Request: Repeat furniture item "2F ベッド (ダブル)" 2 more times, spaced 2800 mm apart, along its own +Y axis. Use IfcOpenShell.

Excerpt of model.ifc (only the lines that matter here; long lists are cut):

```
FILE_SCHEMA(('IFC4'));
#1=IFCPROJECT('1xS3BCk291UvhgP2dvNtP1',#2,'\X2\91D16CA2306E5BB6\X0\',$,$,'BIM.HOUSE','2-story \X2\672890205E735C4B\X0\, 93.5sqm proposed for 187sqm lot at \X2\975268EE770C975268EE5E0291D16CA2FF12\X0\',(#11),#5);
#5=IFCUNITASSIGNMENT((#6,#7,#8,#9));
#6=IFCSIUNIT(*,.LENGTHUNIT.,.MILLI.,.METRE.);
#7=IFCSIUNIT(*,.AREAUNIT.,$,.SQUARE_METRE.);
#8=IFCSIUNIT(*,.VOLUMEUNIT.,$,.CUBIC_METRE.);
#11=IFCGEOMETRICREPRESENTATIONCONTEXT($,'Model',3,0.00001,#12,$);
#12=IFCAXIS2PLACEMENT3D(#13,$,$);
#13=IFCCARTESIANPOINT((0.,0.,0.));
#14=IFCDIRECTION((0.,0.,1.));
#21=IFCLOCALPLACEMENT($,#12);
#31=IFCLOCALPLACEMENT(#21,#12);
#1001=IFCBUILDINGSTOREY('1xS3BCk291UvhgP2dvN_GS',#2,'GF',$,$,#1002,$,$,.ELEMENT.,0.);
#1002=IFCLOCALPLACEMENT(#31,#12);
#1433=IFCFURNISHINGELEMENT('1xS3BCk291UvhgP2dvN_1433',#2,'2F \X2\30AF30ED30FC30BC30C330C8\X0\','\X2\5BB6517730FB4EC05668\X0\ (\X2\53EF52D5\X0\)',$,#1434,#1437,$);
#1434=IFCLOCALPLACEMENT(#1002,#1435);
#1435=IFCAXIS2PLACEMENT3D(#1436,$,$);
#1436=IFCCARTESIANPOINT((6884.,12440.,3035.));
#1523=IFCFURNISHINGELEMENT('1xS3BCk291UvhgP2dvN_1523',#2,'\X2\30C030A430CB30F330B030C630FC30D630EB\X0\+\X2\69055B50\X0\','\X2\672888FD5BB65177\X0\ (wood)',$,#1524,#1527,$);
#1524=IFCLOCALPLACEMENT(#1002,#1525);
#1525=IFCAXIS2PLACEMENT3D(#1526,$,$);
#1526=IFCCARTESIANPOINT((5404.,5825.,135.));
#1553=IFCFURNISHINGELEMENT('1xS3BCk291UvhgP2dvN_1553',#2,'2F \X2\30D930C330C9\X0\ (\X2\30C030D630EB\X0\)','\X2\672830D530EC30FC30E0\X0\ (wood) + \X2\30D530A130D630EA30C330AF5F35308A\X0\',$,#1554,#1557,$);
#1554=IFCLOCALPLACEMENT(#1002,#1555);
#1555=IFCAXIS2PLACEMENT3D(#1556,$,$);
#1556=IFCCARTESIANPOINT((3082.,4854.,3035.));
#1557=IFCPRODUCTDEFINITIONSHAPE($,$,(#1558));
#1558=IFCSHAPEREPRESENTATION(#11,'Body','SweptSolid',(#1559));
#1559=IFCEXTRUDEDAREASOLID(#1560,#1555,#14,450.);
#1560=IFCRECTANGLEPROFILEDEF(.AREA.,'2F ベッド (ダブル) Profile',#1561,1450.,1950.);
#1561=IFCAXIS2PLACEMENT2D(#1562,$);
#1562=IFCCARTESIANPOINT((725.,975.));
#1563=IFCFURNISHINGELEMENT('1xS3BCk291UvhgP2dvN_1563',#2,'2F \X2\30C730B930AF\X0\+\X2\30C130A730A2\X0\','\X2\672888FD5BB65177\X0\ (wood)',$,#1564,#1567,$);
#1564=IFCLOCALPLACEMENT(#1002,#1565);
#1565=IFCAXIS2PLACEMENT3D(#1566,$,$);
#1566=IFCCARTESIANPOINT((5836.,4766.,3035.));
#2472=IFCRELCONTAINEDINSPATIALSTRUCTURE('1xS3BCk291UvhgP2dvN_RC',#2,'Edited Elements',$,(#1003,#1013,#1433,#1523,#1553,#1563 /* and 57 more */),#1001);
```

```python
import ifcopenshell
import ifcopenshell.api.geometry
import ifcopenshell.api.root
import ifcopenshell.util.element
import ifcopenshell.util.placement
import ifcopenshell.util.unit

model = ifcopenshell.open("model.ifc")
unit_scale = ifcopenshell.util.unit.calculate_unit_scale(model)


def reuse_history(source, copy):
    """copy_class also copies each property set's owner history, people and application; keep the originals."""
    for rel in copy.IsDefinedBy:
        if rel.is_a("IfcRelDefinesByProperties") and (history := rel.RelatingPropertyDefinition.OwnerHistory):
            rel.RelatingPropertyDefinition.OwnerHistory = source.OwnerHistory
            ifcopenshell.util.element.remove_deep2(model, history)


source = model.by_guid("1xS3BCk291UvhgP2dvN_1553")
base = ifcopenshell.util.placement.get_local_placement(source.ObjectPlacement)
step = base[:3, 1] * 2.8 / unit_scale

for i in range(1, 3):
    copy = ifcopenshell.api.root.copy_class(model, product=source)
    copy.Representation = ifcopenshell.util.element.copy_deep(
        model, source.Representation, exclude=["IfcGeometricRepresentationContext", "IfcRepresentationMap"]
    )
    reuse_history(source, copy)
    matrix = base.copy()
    matrix[:3, 3] += i * step
    print("added at", matrix[:3, 3].round(3) + 0.0)
    ifcopenshell.api.geometry.edit_object_placement(model, product=copy, matrix=matrix, is_si=False)

model.write("model_v2.ifc")
```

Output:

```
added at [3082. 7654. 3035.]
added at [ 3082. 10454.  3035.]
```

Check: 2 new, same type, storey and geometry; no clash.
